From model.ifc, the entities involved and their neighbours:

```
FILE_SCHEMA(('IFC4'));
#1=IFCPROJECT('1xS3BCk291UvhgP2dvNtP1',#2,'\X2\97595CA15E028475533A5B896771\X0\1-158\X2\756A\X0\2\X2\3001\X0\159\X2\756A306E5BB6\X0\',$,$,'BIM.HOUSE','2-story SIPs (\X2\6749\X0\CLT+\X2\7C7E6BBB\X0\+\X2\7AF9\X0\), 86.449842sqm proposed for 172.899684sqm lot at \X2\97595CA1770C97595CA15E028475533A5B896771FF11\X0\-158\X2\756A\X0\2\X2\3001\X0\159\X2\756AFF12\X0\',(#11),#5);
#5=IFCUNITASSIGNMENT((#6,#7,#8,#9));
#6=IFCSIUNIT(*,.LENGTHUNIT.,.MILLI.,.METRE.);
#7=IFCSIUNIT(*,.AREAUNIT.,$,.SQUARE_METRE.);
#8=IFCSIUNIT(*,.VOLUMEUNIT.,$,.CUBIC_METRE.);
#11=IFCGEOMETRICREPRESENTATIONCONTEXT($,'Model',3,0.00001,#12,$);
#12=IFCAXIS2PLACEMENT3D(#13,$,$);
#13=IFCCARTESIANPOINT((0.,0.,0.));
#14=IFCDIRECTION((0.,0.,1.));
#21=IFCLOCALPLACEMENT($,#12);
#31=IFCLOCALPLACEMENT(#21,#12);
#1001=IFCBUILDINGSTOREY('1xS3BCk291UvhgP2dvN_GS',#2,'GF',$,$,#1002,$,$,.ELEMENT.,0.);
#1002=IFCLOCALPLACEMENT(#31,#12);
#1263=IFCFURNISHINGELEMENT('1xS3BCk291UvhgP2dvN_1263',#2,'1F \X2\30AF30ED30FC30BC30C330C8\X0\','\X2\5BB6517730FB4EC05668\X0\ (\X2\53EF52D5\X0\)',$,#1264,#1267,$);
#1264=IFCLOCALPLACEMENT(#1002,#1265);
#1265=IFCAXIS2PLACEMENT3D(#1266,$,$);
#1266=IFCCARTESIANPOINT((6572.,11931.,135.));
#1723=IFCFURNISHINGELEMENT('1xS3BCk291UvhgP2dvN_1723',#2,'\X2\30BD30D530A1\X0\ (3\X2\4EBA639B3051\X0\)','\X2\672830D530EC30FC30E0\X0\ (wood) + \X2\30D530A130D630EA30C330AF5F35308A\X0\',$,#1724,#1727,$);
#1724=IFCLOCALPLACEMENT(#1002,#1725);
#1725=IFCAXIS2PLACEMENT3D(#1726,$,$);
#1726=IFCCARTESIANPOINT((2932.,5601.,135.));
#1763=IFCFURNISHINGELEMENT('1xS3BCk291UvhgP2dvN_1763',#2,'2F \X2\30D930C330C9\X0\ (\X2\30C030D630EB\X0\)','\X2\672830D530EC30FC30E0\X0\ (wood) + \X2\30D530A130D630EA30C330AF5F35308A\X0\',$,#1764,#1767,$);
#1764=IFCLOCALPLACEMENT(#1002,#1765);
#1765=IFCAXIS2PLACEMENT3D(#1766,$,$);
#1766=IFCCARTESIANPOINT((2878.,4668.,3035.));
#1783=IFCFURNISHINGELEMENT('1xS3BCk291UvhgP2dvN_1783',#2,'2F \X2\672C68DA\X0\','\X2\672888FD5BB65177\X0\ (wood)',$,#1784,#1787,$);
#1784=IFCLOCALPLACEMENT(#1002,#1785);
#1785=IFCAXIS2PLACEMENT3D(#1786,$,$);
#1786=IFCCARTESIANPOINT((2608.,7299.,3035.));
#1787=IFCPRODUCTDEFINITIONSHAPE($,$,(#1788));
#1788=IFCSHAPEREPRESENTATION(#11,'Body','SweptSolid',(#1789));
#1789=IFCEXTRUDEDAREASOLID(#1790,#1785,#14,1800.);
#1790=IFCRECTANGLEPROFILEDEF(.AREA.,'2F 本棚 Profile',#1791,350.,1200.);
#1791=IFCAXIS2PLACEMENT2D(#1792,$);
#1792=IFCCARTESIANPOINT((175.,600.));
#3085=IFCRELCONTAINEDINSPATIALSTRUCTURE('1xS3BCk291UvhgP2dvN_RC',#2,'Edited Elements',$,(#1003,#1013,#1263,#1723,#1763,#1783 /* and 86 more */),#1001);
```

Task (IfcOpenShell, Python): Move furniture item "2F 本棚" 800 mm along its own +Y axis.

```python
import ifcopenshell
import ifcopenshell.api.geometry
import ifcopenshell.util.placement
import ifcopenshell.util.unit

model = ifcopenshell.open("model.ifc")
unit_scale = ifcopenshell.util.unit.calculate_unit_scale(model)

item = model.by_guid("1xS3BCk291UvhgP2dvN_1783")
matrix = ifcopenshell.util.placement.get_local_placement(item.ObjectPlacement)
matrix[:3, 3] += matrix[:3, 1] * 0.8 / unit_scale
ifcopenshell.api.geometry.edit_object_placement(model, product=item, matrix=matrix, is_si=False)

print(ifcopenshell.util.placement.get_local_placement(item.ObjectPlacement).round(3) + 0.0)

model.write("model_edited.ifc")
```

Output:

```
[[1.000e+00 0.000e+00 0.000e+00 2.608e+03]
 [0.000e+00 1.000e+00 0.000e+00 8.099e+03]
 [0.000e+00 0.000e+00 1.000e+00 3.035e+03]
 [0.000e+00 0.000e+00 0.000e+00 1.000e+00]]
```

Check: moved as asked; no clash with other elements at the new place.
